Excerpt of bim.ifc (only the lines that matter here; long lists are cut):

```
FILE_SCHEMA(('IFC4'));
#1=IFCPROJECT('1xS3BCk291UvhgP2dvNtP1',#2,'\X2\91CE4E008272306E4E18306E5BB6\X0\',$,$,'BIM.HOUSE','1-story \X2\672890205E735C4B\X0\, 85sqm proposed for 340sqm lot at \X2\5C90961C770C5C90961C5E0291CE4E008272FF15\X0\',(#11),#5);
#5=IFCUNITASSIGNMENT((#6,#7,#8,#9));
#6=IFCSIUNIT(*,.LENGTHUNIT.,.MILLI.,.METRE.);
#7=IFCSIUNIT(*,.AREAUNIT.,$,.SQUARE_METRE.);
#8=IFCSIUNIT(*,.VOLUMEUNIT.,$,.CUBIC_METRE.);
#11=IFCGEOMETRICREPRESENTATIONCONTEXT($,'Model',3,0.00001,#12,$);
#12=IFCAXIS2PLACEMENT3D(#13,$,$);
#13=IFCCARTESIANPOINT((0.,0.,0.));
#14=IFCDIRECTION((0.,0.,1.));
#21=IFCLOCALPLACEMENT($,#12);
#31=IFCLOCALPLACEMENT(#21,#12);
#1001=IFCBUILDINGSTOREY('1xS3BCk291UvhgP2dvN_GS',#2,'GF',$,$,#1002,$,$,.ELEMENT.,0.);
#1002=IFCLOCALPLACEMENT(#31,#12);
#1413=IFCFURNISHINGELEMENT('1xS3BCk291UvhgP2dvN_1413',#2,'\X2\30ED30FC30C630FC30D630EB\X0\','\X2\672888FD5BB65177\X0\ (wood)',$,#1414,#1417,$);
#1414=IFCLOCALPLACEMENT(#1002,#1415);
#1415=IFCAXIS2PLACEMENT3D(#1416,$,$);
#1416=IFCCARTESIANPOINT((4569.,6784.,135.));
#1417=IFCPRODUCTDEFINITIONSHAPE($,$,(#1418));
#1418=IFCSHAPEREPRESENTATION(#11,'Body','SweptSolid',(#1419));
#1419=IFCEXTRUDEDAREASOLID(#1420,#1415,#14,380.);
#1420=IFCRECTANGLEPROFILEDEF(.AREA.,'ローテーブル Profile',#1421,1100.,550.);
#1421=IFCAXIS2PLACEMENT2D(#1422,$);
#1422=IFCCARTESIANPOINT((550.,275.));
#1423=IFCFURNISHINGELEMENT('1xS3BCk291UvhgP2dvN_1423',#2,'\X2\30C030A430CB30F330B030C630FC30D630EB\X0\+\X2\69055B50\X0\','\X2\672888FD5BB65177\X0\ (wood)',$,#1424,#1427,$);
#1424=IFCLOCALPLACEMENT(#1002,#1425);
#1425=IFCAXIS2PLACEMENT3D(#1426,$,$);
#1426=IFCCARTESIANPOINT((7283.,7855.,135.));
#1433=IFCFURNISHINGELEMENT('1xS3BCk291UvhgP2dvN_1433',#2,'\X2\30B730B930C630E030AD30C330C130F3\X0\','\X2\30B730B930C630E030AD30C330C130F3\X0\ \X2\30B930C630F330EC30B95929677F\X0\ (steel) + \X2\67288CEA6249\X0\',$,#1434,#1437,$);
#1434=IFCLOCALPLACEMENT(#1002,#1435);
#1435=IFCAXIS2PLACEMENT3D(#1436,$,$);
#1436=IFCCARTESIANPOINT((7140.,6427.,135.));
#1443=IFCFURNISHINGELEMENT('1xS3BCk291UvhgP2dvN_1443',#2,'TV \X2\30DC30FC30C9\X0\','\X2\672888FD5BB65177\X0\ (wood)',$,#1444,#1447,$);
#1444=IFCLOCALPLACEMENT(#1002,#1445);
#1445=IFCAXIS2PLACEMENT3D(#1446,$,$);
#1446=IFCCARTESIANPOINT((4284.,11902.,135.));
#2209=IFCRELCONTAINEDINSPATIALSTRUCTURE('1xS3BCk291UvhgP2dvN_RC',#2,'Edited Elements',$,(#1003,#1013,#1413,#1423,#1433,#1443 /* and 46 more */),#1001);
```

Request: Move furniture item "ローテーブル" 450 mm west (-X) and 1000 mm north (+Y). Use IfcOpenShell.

```python
import ifcopenshell
import ifcopenshell.api.geometry
import ifcopenshell.util.placement

model = ifcopenshell.open("bim.ifc")

item = model.by_guid("1xS3BCk291UvhgP2dvN_1413")
matrix = ifcopenshell.util.placement.get_local_placement(item.ObjectPlacement)
matrix[0, 3] -= 450.0
matrix[1, 3] += 1000.0
ifcopenshell.api.geometry.edit_object_placement(model, product=item, matrix=matrix, is_si=False)

print(ifcopenshell.util.placement.get_local_placement(item.ObjectPlacement).round(3) + 0.0)

model.write("bim-out.ifc")
```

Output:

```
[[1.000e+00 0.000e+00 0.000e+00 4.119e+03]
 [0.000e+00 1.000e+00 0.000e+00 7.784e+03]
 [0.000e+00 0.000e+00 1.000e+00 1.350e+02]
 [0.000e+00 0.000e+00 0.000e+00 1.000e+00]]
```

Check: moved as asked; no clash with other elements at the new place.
